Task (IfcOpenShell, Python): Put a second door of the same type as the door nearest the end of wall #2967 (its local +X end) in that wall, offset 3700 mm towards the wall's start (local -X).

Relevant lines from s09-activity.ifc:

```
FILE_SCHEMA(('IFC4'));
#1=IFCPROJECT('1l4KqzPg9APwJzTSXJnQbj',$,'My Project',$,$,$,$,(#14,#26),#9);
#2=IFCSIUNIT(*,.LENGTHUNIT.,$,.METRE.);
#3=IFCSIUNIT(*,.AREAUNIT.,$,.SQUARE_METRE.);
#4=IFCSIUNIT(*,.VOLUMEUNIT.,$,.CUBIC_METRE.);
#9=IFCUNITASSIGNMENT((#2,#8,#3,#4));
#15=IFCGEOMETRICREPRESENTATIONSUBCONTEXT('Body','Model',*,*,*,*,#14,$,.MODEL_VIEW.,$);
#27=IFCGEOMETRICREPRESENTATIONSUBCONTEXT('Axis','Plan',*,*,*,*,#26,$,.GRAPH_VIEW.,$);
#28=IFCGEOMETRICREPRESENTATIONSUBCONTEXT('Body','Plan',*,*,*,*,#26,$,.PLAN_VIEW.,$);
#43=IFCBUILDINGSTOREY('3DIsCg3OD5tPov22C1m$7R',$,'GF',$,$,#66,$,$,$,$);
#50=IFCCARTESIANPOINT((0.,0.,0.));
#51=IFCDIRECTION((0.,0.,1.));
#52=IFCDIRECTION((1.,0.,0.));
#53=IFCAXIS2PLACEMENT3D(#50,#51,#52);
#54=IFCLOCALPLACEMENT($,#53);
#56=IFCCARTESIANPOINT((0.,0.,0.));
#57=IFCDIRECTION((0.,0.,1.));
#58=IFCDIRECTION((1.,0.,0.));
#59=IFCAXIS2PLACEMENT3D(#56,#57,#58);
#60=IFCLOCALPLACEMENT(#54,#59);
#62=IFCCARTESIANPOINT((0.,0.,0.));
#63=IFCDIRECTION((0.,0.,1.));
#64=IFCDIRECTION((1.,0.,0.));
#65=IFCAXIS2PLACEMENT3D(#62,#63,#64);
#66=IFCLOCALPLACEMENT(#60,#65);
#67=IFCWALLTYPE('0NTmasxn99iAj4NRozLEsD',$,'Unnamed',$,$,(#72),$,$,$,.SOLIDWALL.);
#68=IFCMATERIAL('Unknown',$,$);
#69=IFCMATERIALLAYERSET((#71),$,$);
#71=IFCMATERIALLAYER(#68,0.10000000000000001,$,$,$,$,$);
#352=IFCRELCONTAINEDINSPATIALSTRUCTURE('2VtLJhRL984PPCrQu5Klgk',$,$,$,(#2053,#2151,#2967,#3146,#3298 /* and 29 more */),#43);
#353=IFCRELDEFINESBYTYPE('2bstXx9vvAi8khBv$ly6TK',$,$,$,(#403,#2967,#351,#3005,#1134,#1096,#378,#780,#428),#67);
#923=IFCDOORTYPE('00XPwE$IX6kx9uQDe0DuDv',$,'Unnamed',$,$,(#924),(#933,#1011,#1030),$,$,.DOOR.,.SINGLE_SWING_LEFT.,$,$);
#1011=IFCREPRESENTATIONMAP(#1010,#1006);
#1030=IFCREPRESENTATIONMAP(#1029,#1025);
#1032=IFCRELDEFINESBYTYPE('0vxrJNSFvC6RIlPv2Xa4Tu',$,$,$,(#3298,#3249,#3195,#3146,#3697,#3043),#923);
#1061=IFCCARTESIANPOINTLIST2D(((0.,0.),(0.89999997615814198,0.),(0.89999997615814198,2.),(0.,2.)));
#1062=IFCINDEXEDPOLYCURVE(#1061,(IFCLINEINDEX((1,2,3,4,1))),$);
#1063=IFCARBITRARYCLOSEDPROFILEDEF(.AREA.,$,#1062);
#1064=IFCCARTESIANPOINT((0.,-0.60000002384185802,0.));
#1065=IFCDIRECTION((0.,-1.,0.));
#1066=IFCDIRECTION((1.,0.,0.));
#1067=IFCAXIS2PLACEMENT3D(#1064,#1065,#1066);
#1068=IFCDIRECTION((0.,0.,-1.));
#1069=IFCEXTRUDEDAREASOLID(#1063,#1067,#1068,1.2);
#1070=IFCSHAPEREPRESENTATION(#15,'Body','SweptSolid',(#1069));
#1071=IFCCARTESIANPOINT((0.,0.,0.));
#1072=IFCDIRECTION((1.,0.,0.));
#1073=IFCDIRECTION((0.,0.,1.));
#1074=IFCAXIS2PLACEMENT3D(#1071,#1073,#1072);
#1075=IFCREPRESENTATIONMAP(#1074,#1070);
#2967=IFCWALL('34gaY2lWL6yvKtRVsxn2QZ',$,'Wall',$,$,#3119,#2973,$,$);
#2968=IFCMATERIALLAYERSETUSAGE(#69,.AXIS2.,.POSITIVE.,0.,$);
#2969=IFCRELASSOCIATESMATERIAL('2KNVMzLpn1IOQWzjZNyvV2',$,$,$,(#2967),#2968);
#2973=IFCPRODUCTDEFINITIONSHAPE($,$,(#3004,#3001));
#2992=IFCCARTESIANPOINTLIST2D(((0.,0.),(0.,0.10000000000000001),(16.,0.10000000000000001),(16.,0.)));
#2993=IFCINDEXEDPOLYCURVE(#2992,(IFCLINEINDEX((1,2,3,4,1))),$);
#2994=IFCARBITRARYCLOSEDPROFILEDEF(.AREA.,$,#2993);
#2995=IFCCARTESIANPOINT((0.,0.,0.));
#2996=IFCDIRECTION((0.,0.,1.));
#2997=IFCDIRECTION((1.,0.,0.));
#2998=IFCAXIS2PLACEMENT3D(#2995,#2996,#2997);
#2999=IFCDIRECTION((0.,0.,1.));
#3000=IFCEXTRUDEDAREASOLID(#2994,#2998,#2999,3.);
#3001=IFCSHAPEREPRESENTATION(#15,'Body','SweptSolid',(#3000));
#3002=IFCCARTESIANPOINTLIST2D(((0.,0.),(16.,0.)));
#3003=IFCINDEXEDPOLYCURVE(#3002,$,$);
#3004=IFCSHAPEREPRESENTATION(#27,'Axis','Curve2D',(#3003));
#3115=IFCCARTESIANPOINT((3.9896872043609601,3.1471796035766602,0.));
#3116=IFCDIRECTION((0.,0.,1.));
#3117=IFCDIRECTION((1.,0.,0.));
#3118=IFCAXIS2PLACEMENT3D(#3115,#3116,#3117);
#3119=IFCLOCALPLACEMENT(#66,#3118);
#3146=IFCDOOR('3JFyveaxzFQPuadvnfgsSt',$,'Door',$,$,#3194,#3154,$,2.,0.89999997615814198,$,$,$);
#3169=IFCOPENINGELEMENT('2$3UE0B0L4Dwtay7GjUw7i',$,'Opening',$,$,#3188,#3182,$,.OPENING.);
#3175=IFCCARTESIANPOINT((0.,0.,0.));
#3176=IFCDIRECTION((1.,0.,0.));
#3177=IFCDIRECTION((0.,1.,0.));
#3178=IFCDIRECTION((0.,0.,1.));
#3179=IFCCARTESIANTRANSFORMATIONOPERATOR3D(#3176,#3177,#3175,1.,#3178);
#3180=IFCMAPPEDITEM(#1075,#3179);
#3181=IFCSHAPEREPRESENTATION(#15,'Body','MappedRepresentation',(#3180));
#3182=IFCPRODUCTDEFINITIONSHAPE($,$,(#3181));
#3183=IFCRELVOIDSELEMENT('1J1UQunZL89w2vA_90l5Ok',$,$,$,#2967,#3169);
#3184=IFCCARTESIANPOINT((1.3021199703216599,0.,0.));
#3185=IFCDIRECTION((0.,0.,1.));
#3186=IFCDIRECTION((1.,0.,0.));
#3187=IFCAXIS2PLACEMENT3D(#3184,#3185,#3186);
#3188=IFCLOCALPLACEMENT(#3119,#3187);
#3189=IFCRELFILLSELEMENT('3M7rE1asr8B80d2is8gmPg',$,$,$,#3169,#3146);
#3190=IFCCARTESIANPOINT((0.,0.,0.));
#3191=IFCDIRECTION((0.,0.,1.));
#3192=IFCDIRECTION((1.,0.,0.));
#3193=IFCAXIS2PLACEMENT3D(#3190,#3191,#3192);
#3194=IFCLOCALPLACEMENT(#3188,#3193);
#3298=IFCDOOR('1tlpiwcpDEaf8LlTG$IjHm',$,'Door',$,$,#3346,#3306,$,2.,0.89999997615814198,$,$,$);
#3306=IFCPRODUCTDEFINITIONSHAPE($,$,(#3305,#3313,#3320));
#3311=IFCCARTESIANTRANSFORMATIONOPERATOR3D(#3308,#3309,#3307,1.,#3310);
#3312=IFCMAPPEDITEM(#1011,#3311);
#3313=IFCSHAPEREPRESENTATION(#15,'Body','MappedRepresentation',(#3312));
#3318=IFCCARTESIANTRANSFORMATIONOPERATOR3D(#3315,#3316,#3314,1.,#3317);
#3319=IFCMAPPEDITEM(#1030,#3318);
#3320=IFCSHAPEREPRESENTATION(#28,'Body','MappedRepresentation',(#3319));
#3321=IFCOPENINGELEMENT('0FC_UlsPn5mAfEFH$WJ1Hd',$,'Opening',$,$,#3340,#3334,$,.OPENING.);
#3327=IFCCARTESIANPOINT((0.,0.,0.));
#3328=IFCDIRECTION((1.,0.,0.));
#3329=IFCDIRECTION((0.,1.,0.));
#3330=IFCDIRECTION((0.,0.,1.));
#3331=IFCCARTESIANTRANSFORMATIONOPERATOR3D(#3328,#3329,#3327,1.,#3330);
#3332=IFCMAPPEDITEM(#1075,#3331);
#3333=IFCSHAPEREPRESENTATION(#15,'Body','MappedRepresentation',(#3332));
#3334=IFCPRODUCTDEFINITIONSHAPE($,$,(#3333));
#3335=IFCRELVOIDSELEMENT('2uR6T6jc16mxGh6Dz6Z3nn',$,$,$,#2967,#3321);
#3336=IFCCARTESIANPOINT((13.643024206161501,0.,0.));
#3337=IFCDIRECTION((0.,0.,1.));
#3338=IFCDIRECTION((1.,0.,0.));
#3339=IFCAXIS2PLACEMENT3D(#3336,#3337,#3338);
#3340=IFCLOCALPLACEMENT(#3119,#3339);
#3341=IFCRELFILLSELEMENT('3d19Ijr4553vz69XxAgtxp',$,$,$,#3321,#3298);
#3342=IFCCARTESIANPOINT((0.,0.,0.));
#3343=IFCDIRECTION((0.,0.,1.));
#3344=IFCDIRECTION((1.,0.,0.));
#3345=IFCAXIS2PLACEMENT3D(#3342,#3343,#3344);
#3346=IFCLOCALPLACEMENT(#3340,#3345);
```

```python
import ifcopenshell
import ifcopenshell.api.feature
import ifcopenshell.api.geometry
import ifcopenshell.api.root
import ifcopenshell.geom
import ifcopenshell.util.element
import ifcopenshell.util.placement
import ifcopenshell.util.shape

model = ifcopenshell.open("s09-activity.ifc")
settings = ifcopenshell.geom.settings()


def volume(element):
    """Net volume in cubic metres, openings subtracted."""
    shape = ifcopenshell.geom.create_shape(settings, element)
    return ifcopenshell.util.shape.get_volume(shape.geometry)


door = model.by_guid("1tlpiwcpDEaf8LlTG$IjHm")
opening = door.FillsVoids[0].RelatingOpeningElement
wall = opening.VoidsElements[0].RelatingBuildingElement
before = volume(wall)
shift = ifcopenshell.util.placement.get_local_placement(wall.ObjectPlacement)[:3, 0] * -3.7

# copy_class copies the void relationship, type, container and properties, but no geometry.
new_opening = ifcopenshell.api.root.copy_class(model, product=opening)
new_opening.Representation = ifcopenshell.util.element.copy_deep(
    model, opening.Representation, exclude=["IfcGeometricRepresentationContext", "IfcRepresentationMap"]
)
new_door = ifcopenshell.api.root.copy_class(model, product=door)
new_door.Representation = ifcopenshell.util.element.copy_deep(
    model, door.Representation, exclude=["IfcGeometricRepresentationContext", "IfcRepresentationMap"]
)
ifcopenshell.api.feature.add_filling(model, opening=new_opening, element=new_door)

for old, new in ((opening, new_opening), (door, new_door)):
    matrix = ifcopenshell.util.placement.get_local_placement(old.ObjectPlacement)
    matrix[:3, 3] += shift
    ifcopenshell.api.geometry.edit_object_placement(model, product=new, matrix=matrix, is_si=False)

after = volume(wall)

print(f"wall volume {before:.3f} -> {after:.3f} m3")

model.write("s09-activity_updated.ifc")
```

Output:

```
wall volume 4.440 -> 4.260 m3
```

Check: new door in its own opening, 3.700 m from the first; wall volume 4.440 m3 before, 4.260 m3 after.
